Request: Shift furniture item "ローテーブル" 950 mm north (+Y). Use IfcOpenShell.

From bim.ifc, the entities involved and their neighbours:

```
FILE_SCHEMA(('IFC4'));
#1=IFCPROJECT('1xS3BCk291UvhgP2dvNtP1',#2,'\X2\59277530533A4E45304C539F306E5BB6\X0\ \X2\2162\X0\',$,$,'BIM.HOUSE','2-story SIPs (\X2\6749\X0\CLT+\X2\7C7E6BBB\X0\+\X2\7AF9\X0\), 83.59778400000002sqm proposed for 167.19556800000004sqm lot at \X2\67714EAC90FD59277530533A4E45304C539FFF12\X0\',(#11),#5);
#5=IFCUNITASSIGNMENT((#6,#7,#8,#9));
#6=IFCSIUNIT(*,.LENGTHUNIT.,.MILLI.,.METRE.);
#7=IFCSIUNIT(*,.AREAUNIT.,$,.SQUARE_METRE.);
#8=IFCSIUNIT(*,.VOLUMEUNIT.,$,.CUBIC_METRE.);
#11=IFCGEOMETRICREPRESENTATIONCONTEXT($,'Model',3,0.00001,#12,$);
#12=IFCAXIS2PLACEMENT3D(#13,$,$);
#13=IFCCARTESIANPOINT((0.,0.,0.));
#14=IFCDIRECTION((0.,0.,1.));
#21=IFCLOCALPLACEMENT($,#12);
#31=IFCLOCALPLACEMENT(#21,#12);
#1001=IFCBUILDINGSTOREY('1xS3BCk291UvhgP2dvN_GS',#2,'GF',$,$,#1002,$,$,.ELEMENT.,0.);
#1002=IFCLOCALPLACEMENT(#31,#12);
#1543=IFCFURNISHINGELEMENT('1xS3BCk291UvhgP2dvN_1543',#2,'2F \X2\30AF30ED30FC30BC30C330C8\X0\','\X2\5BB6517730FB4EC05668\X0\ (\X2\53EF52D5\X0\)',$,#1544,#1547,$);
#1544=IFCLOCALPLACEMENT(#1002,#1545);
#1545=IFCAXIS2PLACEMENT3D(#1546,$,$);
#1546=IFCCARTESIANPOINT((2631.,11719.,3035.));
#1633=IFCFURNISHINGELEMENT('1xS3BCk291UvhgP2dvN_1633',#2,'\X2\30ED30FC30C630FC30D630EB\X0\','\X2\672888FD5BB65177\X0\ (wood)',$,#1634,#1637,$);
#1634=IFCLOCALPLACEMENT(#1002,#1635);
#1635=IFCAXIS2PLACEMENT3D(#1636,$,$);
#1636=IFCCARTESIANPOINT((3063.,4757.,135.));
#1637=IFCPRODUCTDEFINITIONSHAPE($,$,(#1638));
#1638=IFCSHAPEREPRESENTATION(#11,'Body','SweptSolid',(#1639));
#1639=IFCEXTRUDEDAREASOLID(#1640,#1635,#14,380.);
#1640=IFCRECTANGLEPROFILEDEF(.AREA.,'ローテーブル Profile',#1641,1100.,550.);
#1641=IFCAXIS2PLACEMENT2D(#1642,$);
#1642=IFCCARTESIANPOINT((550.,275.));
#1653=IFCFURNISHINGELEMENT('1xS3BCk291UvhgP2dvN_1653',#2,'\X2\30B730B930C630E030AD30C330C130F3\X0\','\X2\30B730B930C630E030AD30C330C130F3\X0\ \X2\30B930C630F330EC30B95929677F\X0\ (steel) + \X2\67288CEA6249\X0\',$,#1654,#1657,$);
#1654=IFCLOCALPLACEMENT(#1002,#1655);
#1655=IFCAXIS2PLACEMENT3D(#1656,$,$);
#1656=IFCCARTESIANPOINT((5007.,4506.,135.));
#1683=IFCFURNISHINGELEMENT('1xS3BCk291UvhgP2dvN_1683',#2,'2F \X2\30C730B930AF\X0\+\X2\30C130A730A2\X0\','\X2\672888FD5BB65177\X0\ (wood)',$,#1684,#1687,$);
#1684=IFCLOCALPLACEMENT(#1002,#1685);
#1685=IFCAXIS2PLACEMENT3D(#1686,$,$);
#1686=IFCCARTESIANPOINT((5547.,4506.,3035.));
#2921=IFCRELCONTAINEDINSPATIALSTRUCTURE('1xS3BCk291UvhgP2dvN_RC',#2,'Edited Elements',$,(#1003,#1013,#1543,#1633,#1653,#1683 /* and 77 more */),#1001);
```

```python
import ifcopenshell
import ifcopenshell.api.geometry
import ifcopenshell.util.placement
import ifcopenshell.util.unit

model = ifcopenshell.open("bim.ifc")
unit_scale = ifcopenshell.util.unit.calculate_unit_scale(model)

item = model.by_id(1633)
matrix = ifcopenshell.util.placement.get_local_placement(item.ObjectPlacement)
matrix[1, 3] += 0.95 / unit_scale
ifcopenshell.api.geometry.edit_object_placement(model, product=item, matrix=matrix, is_si=False)

print(ifcopenshell.util.placement.get_local_placement(item.ObjectPlacement).round(3) + 0.0)

model.write("bim_rev.ifc")
```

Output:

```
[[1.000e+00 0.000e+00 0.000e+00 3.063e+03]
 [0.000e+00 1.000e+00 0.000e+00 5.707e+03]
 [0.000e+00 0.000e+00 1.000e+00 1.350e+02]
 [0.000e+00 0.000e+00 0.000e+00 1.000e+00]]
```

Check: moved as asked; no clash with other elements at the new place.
